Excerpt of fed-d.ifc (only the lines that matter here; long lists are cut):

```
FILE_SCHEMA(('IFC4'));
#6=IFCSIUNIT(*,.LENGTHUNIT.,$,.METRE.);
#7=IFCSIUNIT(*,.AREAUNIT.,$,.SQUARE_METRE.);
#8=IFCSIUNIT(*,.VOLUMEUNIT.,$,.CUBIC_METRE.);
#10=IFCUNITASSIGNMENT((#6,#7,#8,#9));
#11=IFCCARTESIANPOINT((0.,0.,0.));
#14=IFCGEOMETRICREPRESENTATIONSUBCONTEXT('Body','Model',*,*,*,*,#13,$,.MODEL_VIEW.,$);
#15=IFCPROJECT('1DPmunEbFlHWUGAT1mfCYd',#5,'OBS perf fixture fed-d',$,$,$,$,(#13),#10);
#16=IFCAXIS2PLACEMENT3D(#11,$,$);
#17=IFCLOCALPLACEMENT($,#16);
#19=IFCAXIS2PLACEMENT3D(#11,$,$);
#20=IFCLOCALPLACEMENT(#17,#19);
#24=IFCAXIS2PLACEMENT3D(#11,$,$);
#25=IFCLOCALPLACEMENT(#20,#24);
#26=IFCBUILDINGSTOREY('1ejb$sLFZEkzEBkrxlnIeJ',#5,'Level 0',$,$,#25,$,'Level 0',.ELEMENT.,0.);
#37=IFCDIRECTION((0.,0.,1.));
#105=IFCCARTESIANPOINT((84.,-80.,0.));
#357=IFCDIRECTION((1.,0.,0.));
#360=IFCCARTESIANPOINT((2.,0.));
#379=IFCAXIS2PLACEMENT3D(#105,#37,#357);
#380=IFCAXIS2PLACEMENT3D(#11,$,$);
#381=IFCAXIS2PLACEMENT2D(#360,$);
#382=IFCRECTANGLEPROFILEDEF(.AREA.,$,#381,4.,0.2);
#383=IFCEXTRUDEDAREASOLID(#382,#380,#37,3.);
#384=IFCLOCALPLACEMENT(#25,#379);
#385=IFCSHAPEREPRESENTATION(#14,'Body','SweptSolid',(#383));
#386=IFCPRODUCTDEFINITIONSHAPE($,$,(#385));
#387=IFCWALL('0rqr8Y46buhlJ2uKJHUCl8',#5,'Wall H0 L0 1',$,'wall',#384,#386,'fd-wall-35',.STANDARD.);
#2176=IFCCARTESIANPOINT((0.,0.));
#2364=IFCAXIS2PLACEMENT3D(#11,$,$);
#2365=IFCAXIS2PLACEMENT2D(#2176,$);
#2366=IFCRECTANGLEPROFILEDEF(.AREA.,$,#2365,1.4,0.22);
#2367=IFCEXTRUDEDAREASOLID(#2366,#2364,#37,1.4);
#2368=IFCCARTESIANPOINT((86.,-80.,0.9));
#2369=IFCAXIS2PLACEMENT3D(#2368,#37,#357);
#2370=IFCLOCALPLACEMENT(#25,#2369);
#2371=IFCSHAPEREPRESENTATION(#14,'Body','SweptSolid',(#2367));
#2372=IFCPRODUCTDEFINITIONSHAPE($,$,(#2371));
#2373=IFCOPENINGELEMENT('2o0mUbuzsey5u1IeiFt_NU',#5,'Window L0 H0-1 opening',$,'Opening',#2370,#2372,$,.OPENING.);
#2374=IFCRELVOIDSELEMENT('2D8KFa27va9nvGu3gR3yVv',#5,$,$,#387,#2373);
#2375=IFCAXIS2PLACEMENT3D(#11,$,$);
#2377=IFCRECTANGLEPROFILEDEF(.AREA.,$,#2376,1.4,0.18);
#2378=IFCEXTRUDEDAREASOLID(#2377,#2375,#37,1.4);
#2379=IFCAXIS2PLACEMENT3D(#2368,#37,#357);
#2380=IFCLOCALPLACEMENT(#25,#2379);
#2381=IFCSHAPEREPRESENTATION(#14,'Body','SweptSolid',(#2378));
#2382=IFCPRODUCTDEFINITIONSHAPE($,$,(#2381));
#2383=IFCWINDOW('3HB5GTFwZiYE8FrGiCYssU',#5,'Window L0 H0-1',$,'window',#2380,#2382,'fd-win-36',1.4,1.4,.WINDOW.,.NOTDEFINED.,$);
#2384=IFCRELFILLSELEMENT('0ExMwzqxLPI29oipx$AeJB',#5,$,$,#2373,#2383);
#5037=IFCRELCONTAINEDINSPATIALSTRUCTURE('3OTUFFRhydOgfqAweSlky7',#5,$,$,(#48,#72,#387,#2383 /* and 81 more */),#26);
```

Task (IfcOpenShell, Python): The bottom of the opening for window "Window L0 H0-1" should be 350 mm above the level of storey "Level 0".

```python
import numpy as np
import ifcopenshell
import ifcopenshell.api.geometry
import ifcopenshell.geom
import ifcopenshell.util.element
import ifcopenshell.util.placement
import ifcopenshell.util.shape
import ifcopenshell.util.unit

model = ifcopenshell.open("fed-d.ifc")
unit_scale = ifcopenshell.util.unit.calculate_unit_scale(model)

window = model.by_id(2383)
opening = window.FillsVoids[0].RelatingOpeningElement
storey = ifcopenshell.util.element.get_container(window, ifc_class="IfcBuildingStorey")
level = ifcopenshell.util.placement.get_local_placement(storey.ObjectPlacement)[2, 3]

# The opening's origin need not be at the sill, so measure its lowest point.
shape = ifcopenshell.geom.create_shape(ifcopenshell.geom.settings(), opening)
bottom = ifcopenshell.util.shape.get_shape_bottom_elevation(shape, shape.geometry) / unit_scale
dz = level + 0.35 / unit_scale - bottom

shift = np.array([0.0, 0.0, dz])
# The window is not placed relative to its opening, so move both.
for product in (opening, window):
    matrix = ifcopenshell.util.placement.get_local_placement(product.ObjectPlacement)
    matrix[:3, 3] += shift
    ifcopenshell.api.geometry.edit_object_placement(model, product=product, matrix=matrix, is_si=False)

print(f"moved by {dz * unit_scale:+.3f} m")

model.write("fed-d_v2.ifc")
```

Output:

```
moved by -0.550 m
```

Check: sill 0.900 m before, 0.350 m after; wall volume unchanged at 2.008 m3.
